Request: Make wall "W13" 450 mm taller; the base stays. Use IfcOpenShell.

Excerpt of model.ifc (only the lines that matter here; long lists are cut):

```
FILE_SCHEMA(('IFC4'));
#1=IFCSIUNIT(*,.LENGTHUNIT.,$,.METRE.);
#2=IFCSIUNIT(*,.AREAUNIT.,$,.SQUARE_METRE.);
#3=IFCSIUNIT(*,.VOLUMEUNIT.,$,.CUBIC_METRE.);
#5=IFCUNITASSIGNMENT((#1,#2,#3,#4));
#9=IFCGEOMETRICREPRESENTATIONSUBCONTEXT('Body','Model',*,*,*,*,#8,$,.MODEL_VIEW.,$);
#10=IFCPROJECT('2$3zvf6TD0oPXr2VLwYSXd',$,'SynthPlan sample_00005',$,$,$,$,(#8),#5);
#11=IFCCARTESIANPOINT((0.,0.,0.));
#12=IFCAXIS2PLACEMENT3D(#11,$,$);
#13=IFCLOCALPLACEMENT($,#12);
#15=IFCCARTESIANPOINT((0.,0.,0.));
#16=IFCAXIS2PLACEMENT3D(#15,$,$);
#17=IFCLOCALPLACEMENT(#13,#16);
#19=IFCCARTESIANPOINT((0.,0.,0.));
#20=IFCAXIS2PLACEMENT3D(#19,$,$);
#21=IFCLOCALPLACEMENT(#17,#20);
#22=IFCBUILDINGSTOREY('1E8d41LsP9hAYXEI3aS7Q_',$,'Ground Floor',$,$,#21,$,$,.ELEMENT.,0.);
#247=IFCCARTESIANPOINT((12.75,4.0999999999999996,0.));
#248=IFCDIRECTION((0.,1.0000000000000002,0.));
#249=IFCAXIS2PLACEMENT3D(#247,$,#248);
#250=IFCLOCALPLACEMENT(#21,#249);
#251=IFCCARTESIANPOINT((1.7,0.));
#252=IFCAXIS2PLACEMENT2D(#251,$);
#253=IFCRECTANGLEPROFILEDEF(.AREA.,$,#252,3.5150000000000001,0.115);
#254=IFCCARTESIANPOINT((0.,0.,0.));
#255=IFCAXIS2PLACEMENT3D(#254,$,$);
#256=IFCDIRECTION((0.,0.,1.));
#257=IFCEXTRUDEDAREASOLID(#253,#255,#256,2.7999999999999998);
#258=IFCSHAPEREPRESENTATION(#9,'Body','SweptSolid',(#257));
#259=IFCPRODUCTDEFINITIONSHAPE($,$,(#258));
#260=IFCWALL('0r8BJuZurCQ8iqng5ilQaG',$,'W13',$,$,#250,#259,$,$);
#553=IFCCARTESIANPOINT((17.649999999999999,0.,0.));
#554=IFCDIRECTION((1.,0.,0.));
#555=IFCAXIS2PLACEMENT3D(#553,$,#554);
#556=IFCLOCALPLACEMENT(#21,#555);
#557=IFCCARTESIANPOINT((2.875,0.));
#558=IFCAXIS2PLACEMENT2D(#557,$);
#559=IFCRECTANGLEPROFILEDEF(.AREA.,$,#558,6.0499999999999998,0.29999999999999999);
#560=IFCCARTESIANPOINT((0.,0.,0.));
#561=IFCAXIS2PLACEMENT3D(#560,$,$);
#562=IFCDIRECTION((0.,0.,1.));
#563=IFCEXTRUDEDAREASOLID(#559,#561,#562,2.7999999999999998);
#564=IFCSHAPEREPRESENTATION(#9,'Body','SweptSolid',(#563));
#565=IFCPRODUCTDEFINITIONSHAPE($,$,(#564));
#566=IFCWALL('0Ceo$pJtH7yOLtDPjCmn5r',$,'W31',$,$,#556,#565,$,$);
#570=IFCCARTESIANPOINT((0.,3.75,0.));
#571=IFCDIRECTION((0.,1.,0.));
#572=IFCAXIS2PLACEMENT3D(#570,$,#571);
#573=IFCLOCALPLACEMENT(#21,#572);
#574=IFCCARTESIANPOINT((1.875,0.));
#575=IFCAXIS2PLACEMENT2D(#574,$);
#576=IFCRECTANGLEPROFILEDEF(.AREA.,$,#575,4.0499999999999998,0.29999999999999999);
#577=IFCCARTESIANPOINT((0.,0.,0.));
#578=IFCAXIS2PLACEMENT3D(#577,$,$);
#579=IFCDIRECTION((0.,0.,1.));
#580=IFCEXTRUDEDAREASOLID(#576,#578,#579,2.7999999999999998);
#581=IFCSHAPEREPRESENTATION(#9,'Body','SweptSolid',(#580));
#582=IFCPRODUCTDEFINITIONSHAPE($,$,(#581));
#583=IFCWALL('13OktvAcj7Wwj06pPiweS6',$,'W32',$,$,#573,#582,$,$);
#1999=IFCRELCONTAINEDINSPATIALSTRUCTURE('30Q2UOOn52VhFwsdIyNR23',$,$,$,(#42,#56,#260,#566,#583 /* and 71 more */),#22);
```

```python
import ifcopenshell
import ifcopenshell.geom
import ifcopenshell.util.representation
import ifcopenshell.util.shape
import ifcopenshell.util.unit

model = ifcopenshell.open("model.ifc")
unit_scale = ifcopenshell.util.unit.calculate_unit_scale(model)
settings = ifcopenshell.geom.settings()


def volume(element):
    """Net volume in cubic metres, openings subtracted."""
    shape = ifcopenshell.geom.create_shape(settings, element)
    return ifcopenshell.util.shape.get_volume(shape.geometry)


wall = model.by_guid("0r8BJuZurCQ8iqng5ilQaG")
before = volume(wall)

body = ifcopenshell.util.representation.get_representation(wall, "Model", "Body")
solid = body.Items[0]
old_height = solid.Depth
solid.Depth += 0.45 / unit_scale
after = volume(wall)

print(f"height {old_height:g} -> {solid.Depth:g}, volume {before:.3f} -> {after:.3f} m3")

model.write("model_updated.ifc")
```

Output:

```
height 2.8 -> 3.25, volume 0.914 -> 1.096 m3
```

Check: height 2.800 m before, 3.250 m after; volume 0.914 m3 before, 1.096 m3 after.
